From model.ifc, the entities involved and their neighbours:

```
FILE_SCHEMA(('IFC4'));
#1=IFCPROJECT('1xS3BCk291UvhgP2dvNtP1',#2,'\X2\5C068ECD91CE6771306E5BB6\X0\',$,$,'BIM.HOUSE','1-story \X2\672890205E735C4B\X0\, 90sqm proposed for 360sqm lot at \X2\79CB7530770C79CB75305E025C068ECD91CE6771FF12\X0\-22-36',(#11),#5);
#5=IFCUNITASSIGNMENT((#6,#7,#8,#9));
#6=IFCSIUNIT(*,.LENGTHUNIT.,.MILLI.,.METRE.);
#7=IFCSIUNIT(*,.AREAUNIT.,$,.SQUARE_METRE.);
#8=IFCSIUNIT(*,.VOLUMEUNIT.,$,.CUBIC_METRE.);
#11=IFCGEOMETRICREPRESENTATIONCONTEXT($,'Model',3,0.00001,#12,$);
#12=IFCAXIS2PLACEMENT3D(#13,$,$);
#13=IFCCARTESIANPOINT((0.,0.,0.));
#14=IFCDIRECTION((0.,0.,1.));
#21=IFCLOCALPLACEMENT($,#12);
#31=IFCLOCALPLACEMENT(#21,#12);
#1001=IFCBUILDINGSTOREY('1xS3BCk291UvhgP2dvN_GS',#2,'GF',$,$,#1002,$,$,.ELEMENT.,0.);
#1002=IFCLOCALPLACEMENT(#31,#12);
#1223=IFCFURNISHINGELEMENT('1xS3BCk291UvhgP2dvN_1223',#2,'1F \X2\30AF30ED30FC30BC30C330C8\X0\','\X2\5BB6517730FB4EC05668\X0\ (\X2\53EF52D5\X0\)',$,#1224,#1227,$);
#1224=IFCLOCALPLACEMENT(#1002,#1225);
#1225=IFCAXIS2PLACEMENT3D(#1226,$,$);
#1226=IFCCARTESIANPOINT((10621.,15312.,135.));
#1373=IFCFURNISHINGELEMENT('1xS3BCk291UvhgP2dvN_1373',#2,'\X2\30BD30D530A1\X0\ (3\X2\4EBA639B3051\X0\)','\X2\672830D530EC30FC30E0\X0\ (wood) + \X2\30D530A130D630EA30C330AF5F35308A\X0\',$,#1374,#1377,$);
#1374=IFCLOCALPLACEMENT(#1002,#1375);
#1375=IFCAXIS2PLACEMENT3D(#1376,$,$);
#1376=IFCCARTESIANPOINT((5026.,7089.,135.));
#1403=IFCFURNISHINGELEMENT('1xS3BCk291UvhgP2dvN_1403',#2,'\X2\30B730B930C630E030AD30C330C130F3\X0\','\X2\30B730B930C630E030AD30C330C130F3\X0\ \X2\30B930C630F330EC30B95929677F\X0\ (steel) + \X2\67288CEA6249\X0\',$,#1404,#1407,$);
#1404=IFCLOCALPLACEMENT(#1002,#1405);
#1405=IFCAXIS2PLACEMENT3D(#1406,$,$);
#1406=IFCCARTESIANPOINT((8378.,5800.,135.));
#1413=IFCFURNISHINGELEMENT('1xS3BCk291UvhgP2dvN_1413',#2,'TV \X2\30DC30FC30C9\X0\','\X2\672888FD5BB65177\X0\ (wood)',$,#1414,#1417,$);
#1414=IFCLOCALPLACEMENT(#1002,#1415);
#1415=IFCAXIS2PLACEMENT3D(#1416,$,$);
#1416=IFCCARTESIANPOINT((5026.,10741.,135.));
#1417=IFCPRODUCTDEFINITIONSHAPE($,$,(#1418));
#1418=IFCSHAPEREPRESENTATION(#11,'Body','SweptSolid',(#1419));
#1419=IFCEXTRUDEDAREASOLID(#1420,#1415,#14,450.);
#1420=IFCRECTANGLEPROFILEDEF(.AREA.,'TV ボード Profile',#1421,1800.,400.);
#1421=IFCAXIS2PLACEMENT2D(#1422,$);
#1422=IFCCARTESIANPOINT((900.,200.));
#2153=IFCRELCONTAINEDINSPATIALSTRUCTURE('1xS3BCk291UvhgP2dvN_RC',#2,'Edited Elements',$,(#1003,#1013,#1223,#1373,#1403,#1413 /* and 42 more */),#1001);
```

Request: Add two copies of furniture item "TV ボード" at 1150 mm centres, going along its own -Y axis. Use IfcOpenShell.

```python
import ifcopenshell
import ifcopenshell.api.geometry
import ifcopenshell.api.root
import ifcopenshell.util.element
import ifcopenshell.util.placement
import ifcopenshell.util.unit

model = ifcopenshell.open("model.ifc")
unit_scale = ifcopenshell.util.unit.calculate_unit_scale(model)


def reuse_history(source, copy):
    """copy_class also copies each property set's owner history, people and application; keep the originals."""
    for rel in copy.IsDefinedBy:
        if rel.is_a("IfcRelDefinesByProperties") and (history := rel.RelatingPropertyDefinition.OwnerHistory):
            rel.RelatingPropertyDefinition.OwnerHistory = source.OwnerHistory
            ifcopenshell.util.element.remove_deep2(model, history)


source = model.by_guid("1xS3BCk291UvhgP2dvN_1413")
base = ifcopenshell.util.placement.get_local_placement(source.ObjectPlacement)
step = -base[:3, 1] * 1.15 / unit_scale

for i in range(1, 3):
    copy = ifcopenshell.api.root.copy_class(model, product=source)
    copy.Representation = ifcopenshell.util.element.copy_deep(
        model, source.Representation, exclude=["IfcGeometricRepresentationContext", "IfcRepresentationMap"]
    )
    reuse_history(source, copy)
    matrix = base.copy()
    matrix[:3, 3] += i * step
    print("added at", matrix[:3, 3].round(3) + 0.0)
    ifcopenshell.api.geometry.edit_object_placement(model, product=copy, matrix=matrix, is_si=False)

model.write("model-out.ifc")
```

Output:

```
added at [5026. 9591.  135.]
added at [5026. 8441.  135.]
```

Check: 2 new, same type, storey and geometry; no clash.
